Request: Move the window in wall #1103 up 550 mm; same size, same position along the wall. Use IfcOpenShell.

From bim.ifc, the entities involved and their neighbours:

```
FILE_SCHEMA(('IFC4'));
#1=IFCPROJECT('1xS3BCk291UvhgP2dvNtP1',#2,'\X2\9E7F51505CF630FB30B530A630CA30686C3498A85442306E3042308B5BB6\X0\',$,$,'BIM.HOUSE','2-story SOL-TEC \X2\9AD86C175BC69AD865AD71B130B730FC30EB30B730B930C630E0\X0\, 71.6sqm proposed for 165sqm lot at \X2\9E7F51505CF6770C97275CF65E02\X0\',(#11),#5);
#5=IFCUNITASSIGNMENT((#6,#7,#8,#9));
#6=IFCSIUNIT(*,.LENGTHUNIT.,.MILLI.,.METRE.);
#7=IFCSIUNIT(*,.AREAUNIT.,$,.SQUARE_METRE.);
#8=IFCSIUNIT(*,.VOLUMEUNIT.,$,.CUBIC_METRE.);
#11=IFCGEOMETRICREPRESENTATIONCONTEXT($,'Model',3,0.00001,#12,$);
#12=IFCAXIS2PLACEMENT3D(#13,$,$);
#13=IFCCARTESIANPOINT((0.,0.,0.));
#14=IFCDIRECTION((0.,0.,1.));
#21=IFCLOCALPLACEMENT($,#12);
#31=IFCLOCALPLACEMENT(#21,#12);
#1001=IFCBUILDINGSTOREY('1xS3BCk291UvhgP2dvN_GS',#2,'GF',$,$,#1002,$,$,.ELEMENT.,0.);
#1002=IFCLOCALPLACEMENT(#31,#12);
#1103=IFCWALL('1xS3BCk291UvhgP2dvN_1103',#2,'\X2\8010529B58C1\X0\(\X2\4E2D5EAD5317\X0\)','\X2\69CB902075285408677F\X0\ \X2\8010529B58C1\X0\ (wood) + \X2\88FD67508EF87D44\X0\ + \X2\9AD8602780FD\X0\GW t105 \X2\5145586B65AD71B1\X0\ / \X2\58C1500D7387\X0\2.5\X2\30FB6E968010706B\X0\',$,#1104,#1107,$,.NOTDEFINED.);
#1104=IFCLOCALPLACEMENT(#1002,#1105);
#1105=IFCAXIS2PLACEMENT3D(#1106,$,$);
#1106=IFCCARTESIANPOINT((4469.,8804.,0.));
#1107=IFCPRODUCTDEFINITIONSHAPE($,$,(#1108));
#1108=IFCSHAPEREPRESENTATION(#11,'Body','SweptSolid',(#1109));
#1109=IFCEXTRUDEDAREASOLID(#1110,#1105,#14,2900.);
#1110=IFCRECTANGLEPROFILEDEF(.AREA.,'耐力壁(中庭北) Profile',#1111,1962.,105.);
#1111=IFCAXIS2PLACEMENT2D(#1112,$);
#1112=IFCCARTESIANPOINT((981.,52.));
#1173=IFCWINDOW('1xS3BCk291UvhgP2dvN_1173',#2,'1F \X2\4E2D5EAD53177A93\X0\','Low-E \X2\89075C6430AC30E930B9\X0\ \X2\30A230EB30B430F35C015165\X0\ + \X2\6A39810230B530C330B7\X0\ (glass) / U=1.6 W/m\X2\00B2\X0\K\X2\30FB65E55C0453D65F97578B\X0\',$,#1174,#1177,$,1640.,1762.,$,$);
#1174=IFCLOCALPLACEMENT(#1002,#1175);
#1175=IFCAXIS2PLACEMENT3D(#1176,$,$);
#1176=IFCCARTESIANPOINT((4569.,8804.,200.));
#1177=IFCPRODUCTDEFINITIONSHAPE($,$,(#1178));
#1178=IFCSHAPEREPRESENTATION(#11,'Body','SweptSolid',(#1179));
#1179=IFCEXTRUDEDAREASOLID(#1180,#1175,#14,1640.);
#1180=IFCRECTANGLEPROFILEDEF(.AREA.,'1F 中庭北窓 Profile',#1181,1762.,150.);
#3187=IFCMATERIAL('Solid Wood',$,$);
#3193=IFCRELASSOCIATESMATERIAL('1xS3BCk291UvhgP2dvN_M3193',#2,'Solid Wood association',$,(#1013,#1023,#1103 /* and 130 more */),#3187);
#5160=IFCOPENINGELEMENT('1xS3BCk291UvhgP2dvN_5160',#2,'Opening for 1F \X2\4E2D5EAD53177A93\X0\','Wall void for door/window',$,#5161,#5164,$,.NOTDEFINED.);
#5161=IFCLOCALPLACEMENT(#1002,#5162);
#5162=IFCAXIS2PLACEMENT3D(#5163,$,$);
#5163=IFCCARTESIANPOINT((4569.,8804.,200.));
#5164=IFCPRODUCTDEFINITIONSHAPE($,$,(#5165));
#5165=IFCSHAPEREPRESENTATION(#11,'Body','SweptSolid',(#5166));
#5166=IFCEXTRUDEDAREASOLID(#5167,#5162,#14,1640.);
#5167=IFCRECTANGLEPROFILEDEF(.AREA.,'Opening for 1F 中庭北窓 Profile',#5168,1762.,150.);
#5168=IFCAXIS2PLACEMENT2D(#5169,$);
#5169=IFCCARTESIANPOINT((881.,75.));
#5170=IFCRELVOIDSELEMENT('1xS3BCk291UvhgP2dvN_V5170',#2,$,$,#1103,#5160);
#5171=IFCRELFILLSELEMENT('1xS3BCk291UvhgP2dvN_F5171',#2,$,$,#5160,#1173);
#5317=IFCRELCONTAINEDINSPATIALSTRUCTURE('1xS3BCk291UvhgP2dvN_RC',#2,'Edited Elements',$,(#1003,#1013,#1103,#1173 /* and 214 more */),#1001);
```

```python
import numpy as np
import ifcopenshell
import ifcopenshell.api.geometry
import ifcopenshell.util.placement
import ifcopenshell.util.unit

model = ifcopenshell.open("bim.ifc")
unit_scale = ifcopenshell.util.unit.calculate_unit_scale(model)

window = model.by_guid("1xS3BCk291UvhgP2dvN_1173")
opening = window.FillsVoids[0].RelatingOpeningElement
dz = 0.55 / unit_scale

shift = np.array([0.0, 0.0, dz])
# The window is not placed relative to its opening, so move both.
for product in (opening, window):
    matrix = ifcopenshell.util.placement.get_local_placement(product.ObjectPlacement)
    matrix[:3, 3] += shift
    ifcopenshell.api.geometry.edit_object_placement(model, product=product, matrix=matrix, is_si=False)

print(f"moved by {dz * unit_scale:+.3f} m")

model.write("bim_rev.ifc")
```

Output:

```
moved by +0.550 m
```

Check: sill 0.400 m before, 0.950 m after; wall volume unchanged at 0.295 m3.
